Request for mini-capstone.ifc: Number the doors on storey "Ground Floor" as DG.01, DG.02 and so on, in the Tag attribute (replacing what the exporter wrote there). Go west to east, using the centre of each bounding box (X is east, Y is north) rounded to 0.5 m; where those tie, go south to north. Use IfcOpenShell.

First a look at what the model holds.

```python
import ifcopenshell
import ifcopenshell.util.element
import ifcopenshell.util.placement

model = ifcopenshell.open("mini-capstone.ifc")
print(model.schema)
storey = next(s for s in model.by_type("IfcBuildingStorey") if s.Name == "Ground Floor")
doors = [e for e in ifcopenshell.util.element.get_decomposition(storey) if e.is_a("IfcDoor")]
for e in sorted(doors, key=lambda e: e.id()):
    origin = ifcopenshell.util.placement.get_local_placement(e.ObjectPlacement)[:3, 3]
    print(e.id(), e.Tag, e.Name, origin.round(2) + 0.0, sep=" | ")
```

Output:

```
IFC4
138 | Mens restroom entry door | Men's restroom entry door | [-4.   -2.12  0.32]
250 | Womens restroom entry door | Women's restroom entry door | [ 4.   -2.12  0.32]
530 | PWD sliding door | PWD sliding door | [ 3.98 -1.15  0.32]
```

```python
import ifcopenshell
import ifcopenshell.geom
import ifcopenshell.util.element
import ifcopenshell.util.shape

model = ifcopenshell.open("mini-capstone.ifc")
settings = ifcopenshell.geom.settings()
settings.set("use-world-coords", True)


def centre(element):
    shape = ifcopenshell.geom.create_shape(settings, element)
    return ifcopenshell.util.shape.get_bbox_centroid(shape.geometry)


storey = next(s for s in model.by_type("IfcBuildingStorey") if s.Name == "Ground Floor")
doors = [e for e in ifcopenshell.util.element.get_decomposition(storey) if e.is_a("IfcDoor")]

# Insertion points can sit at a corner or the storey origin, so sort by the geometry (in metres).
centres = {e: centre(e) for e in doors}
doors.sort(key=lambda e: (round(centres[e][0] / 0.5), centres[e][1]))

for i, e in enumerate(doors, start=1):
    number = f"DG.{i:02d}"
    e.Tag = number
    print(e.id(), number)

model.write("mini-capstone_updated.ifc")
```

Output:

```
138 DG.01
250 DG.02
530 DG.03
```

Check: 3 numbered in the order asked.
